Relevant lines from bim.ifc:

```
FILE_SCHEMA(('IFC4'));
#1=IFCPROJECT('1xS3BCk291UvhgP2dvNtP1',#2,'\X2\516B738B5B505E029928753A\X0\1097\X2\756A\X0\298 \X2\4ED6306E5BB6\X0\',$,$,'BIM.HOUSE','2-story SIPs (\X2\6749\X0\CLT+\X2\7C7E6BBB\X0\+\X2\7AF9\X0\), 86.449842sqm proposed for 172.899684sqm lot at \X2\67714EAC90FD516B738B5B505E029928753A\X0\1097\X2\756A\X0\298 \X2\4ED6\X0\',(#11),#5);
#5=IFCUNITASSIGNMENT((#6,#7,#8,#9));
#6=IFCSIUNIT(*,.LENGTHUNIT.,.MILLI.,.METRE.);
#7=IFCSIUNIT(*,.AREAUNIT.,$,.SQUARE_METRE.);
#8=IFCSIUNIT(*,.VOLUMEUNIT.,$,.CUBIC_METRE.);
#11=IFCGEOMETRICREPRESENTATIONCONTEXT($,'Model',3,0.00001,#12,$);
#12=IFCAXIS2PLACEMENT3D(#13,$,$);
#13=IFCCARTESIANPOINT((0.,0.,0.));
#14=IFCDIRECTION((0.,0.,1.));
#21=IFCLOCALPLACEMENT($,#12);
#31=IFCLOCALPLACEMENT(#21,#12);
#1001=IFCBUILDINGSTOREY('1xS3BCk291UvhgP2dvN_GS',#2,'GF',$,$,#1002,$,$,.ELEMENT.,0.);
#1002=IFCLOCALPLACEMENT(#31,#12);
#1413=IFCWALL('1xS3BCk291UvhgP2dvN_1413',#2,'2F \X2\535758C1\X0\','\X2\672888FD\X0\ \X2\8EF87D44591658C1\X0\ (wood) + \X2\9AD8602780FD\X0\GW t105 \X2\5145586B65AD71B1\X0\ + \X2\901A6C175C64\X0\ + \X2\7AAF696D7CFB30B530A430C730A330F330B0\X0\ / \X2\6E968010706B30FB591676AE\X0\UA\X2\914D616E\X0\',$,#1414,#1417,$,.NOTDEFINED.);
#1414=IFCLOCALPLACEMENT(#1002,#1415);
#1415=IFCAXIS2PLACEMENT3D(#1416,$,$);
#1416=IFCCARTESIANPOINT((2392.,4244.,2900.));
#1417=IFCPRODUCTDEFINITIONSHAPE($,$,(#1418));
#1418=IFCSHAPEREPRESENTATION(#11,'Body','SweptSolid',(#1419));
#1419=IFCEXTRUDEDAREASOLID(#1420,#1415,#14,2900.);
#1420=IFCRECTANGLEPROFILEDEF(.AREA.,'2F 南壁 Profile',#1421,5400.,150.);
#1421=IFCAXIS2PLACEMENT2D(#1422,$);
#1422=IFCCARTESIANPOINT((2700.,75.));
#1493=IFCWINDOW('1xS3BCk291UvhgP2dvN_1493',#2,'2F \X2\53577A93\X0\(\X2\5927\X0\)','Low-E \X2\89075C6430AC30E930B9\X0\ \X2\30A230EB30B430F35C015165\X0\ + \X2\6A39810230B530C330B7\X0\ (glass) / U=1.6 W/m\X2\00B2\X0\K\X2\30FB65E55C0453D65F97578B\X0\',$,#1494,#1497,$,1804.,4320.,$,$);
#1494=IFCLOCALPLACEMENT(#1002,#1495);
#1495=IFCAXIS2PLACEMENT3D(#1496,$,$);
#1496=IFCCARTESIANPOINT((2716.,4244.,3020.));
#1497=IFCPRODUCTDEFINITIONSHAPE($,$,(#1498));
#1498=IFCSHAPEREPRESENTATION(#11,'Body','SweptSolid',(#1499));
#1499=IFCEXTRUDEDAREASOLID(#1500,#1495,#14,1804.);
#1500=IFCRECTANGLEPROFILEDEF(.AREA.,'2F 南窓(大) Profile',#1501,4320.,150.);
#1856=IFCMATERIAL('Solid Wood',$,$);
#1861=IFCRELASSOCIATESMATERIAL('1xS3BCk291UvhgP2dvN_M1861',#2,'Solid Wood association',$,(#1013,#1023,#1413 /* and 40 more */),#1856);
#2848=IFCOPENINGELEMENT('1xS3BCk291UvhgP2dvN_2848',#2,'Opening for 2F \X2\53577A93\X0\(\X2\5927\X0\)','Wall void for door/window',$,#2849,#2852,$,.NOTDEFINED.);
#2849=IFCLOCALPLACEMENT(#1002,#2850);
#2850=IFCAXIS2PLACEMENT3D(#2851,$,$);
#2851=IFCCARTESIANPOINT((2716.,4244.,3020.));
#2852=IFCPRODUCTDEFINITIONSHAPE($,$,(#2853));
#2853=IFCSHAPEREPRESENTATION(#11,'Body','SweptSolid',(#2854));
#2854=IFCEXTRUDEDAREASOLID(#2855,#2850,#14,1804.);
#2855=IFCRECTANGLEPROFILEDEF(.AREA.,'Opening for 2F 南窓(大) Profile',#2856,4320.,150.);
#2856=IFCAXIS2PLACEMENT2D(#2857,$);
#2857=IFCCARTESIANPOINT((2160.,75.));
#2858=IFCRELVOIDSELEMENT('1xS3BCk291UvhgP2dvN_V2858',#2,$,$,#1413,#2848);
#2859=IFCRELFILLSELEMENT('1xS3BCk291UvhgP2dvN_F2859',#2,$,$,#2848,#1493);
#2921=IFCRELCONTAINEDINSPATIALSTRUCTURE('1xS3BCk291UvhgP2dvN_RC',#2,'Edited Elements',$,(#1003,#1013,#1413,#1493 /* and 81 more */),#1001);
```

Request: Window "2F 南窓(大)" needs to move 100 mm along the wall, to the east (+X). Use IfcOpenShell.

```python
import ifcopenshell
import ifcopenshell.api.geometry
import ifcopenshell.util.placement

model = ifcopenshell.open("bim.ifc")

window = model.by_id(1493)
opening = window.FillsVoids[0].RelatingOpeningElement
wall = opening.VoidsElements[0].RelatingBuildingElement

wall_matrix = ifcopenshell.util.placement.get_local_placement(wall.ObjectPlacement)
shift = wall_matrix[:3, 0] * 100.0
before = ifcopenshell.util.placement.get_local_placement(window.ObjectPlacement)[:3, 3].copy()

# The window is not placed relative to its opening, so move both.
for product in (opening, window):
    matrix = ifcopenshell.util.placement.get_local_placement(product.ObjectPlacement)
    matrix[:3, 3] += shift
    ifcopenshell.api.geometry.edit_object_placement(model, product=product, matrix=matrix, is_si=False)

after = ifcopenshell.util.placement.get_local_placement(window.ObjectPlacement)[:3, 3]
print("window moved by", (after - before).round(3) + 0.0)

model.write("bim_rev.ifc")
```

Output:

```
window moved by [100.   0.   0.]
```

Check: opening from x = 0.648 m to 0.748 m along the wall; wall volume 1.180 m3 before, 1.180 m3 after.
